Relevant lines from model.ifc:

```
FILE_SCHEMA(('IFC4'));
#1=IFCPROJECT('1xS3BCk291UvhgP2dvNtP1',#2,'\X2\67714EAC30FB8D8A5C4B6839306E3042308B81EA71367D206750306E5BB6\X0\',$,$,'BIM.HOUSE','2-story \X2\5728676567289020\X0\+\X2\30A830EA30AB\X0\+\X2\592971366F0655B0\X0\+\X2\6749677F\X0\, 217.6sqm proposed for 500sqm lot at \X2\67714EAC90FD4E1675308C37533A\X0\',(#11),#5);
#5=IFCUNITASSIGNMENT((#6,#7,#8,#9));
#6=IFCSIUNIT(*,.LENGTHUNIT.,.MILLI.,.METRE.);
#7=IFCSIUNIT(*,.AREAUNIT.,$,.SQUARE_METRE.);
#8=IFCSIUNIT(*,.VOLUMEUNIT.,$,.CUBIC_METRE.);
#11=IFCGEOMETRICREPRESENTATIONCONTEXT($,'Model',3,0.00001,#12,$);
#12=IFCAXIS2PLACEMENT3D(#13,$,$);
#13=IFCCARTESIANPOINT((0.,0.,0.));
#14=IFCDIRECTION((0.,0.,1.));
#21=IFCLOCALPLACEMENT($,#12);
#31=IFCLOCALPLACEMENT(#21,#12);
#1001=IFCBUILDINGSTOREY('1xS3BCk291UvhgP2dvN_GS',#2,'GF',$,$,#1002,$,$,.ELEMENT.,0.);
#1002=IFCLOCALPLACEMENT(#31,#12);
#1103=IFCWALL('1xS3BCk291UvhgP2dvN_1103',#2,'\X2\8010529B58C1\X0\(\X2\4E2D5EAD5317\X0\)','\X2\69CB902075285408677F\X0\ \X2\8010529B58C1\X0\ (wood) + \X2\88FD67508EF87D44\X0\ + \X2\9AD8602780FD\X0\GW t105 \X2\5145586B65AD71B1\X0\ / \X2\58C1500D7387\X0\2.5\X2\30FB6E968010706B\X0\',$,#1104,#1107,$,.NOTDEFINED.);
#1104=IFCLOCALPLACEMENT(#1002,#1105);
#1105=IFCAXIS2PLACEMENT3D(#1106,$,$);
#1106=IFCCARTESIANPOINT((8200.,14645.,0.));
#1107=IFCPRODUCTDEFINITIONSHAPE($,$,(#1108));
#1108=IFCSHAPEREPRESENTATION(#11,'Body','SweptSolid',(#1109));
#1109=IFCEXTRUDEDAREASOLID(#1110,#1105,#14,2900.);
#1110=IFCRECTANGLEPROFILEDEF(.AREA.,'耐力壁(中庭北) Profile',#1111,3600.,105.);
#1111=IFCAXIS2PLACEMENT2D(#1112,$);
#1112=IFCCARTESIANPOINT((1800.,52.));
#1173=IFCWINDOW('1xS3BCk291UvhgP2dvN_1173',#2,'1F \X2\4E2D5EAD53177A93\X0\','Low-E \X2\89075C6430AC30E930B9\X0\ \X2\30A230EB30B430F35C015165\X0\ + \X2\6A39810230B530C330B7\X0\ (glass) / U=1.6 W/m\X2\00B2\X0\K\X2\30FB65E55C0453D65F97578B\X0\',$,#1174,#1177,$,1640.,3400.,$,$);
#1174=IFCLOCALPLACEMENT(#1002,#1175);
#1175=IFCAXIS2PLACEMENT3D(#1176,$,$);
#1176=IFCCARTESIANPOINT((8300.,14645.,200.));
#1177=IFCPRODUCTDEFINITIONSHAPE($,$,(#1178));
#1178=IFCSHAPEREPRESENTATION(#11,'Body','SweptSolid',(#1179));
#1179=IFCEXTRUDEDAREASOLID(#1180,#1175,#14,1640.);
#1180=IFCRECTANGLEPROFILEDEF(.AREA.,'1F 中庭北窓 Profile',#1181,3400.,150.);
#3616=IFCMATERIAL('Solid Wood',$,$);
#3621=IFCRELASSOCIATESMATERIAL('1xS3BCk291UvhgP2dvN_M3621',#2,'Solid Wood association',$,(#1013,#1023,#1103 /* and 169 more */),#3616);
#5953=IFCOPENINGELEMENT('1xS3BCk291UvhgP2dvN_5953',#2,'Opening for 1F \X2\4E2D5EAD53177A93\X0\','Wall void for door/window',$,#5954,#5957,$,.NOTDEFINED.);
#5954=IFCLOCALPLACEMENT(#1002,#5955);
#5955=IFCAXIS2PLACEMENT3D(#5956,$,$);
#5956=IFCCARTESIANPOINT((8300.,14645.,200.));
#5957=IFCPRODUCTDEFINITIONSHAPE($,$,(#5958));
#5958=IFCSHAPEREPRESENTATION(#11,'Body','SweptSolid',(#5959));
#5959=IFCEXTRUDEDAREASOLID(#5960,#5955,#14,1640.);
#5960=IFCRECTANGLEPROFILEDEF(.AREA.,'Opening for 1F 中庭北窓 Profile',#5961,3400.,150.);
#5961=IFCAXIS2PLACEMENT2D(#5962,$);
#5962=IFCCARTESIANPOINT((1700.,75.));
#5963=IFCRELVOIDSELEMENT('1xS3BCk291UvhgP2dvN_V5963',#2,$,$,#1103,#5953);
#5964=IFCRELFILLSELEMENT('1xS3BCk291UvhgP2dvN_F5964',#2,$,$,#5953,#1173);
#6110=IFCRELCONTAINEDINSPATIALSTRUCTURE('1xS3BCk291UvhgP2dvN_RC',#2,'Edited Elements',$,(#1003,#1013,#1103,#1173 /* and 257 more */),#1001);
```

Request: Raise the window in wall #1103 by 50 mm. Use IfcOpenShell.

```python
import numpy as np
import ifcopenshell
import ifcopenshell.api.geometry
import ifcopenshell.util.placement
import ifcopenshell.util.unit

model = ifcopenshell.open("model.ifc")
unit_scale = ifcopenshell.util.unit.calculate_unit_scale(model)

window = model.by_id(1173)
opening = window.FillsVoids[0].RelatingOpeningElement
dz = 50.0

shift = np.array([0.0, 0.0, dz])
# The window is not placed relative to its opening, so move both.
for product in (opening, window):
    matrix = ifcopenshell.util.placement.get_local_placement(product.ObjectPlacement)
    matrix[:3, 3] += shift
    ifcopenshell.api.geometry.edit_object_placement(model, product=product, matrix=matrix, is_si=False)

print(f"moved by {dz * unit_scale:+.3f} m")

model.write("model_v2.ifc")
```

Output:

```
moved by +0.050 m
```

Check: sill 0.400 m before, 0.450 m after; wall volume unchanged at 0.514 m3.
